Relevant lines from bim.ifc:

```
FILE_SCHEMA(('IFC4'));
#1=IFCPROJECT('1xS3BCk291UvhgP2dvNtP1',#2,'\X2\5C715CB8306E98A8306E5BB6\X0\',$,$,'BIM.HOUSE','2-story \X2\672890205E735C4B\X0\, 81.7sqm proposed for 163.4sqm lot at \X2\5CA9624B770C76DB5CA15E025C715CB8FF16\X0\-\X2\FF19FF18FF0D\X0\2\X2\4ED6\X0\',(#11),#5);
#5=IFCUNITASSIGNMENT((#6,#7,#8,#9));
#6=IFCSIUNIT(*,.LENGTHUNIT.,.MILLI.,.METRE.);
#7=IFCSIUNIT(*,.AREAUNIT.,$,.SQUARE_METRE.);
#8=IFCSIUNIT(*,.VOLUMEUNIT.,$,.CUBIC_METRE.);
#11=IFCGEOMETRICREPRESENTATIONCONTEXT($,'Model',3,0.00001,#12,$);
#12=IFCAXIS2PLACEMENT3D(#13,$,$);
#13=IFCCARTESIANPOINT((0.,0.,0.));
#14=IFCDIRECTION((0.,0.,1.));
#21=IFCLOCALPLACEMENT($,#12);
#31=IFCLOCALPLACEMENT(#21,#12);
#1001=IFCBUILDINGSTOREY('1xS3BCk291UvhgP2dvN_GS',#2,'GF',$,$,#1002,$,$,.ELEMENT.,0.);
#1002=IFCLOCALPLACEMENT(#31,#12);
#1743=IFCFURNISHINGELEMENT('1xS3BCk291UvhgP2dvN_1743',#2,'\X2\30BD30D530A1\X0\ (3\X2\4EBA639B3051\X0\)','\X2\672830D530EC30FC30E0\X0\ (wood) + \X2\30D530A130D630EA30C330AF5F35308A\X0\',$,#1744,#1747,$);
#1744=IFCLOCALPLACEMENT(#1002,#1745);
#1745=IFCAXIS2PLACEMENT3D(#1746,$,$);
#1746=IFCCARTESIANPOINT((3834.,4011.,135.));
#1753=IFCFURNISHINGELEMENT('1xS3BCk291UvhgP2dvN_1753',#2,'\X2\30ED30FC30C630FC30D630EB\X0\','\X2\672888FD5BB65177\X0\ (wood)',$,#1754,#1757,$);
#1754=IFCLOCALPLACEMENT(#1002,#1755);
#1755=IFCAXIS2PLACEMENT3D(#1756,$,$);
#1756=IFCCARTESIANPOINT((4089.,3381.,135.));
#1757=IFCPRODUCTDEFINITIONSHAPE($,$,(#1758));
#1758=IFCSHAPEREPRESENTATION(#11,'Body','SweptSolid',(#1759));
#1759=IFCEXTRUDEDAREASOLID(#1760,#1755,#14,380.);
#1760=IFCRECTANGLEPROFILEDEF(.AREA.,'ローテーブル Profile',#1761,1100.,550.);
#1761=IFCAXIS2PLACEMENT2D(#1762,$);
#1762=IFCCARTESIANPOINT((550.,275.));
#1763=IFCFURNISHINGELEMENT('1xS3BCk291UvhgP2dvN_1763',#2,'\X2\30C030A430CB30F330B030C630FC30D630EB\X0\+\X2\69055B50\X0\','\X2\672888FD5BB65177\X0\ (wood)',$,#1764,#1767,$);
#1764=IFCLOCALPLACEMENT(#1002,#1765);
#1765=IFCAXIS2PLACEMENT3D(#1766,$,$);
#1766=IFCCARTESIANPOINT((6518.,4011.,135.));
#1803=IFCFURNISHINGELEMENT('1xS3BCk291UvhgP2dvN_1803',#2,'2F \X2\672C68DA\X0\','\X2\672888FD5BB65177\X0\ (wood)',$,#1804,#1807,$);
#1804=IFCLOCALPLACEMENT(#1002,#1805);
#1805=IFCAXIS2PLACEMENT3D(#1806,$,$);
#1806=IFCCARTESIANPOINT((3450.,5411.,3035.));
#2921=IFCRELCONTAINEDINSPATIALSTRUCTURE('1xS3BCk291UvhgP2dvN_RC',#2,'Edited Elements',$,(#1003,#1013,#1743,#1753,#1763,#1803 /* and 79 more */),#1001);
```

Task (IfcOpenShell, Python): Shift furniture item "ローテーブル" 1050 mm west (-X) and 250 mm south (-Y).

```python
import ifcopenshell
import ifcopenshell.api.geometry
import ifcopenshell.util.placement

model = ifcopenshell.open("bim.ifc")

item = model.by_id(1753)
matrix = ifcopenshell.util.placement.get_local_placement(item.ObjectPlacement)
matrix[0, 3] -= 1050.0
matrix[1, 3] -= 250.0
ifcopenshell.api.geometry.edit_object_placement(model, product=item, matrix=matrix, is_si=False)

print(ifcopenshell.util.placement.get_local_placement(item.ObjectPlacement).round(3) + 0.0)

model.write("bim-out.ifc")
```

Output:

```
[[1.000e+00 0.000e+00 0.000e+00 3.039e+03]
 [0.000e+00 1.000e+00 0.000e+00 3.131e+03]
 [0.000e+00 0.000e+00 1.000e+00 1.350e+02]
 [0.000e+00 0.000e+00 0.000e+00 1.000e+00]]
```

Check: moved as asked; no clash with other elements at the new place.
